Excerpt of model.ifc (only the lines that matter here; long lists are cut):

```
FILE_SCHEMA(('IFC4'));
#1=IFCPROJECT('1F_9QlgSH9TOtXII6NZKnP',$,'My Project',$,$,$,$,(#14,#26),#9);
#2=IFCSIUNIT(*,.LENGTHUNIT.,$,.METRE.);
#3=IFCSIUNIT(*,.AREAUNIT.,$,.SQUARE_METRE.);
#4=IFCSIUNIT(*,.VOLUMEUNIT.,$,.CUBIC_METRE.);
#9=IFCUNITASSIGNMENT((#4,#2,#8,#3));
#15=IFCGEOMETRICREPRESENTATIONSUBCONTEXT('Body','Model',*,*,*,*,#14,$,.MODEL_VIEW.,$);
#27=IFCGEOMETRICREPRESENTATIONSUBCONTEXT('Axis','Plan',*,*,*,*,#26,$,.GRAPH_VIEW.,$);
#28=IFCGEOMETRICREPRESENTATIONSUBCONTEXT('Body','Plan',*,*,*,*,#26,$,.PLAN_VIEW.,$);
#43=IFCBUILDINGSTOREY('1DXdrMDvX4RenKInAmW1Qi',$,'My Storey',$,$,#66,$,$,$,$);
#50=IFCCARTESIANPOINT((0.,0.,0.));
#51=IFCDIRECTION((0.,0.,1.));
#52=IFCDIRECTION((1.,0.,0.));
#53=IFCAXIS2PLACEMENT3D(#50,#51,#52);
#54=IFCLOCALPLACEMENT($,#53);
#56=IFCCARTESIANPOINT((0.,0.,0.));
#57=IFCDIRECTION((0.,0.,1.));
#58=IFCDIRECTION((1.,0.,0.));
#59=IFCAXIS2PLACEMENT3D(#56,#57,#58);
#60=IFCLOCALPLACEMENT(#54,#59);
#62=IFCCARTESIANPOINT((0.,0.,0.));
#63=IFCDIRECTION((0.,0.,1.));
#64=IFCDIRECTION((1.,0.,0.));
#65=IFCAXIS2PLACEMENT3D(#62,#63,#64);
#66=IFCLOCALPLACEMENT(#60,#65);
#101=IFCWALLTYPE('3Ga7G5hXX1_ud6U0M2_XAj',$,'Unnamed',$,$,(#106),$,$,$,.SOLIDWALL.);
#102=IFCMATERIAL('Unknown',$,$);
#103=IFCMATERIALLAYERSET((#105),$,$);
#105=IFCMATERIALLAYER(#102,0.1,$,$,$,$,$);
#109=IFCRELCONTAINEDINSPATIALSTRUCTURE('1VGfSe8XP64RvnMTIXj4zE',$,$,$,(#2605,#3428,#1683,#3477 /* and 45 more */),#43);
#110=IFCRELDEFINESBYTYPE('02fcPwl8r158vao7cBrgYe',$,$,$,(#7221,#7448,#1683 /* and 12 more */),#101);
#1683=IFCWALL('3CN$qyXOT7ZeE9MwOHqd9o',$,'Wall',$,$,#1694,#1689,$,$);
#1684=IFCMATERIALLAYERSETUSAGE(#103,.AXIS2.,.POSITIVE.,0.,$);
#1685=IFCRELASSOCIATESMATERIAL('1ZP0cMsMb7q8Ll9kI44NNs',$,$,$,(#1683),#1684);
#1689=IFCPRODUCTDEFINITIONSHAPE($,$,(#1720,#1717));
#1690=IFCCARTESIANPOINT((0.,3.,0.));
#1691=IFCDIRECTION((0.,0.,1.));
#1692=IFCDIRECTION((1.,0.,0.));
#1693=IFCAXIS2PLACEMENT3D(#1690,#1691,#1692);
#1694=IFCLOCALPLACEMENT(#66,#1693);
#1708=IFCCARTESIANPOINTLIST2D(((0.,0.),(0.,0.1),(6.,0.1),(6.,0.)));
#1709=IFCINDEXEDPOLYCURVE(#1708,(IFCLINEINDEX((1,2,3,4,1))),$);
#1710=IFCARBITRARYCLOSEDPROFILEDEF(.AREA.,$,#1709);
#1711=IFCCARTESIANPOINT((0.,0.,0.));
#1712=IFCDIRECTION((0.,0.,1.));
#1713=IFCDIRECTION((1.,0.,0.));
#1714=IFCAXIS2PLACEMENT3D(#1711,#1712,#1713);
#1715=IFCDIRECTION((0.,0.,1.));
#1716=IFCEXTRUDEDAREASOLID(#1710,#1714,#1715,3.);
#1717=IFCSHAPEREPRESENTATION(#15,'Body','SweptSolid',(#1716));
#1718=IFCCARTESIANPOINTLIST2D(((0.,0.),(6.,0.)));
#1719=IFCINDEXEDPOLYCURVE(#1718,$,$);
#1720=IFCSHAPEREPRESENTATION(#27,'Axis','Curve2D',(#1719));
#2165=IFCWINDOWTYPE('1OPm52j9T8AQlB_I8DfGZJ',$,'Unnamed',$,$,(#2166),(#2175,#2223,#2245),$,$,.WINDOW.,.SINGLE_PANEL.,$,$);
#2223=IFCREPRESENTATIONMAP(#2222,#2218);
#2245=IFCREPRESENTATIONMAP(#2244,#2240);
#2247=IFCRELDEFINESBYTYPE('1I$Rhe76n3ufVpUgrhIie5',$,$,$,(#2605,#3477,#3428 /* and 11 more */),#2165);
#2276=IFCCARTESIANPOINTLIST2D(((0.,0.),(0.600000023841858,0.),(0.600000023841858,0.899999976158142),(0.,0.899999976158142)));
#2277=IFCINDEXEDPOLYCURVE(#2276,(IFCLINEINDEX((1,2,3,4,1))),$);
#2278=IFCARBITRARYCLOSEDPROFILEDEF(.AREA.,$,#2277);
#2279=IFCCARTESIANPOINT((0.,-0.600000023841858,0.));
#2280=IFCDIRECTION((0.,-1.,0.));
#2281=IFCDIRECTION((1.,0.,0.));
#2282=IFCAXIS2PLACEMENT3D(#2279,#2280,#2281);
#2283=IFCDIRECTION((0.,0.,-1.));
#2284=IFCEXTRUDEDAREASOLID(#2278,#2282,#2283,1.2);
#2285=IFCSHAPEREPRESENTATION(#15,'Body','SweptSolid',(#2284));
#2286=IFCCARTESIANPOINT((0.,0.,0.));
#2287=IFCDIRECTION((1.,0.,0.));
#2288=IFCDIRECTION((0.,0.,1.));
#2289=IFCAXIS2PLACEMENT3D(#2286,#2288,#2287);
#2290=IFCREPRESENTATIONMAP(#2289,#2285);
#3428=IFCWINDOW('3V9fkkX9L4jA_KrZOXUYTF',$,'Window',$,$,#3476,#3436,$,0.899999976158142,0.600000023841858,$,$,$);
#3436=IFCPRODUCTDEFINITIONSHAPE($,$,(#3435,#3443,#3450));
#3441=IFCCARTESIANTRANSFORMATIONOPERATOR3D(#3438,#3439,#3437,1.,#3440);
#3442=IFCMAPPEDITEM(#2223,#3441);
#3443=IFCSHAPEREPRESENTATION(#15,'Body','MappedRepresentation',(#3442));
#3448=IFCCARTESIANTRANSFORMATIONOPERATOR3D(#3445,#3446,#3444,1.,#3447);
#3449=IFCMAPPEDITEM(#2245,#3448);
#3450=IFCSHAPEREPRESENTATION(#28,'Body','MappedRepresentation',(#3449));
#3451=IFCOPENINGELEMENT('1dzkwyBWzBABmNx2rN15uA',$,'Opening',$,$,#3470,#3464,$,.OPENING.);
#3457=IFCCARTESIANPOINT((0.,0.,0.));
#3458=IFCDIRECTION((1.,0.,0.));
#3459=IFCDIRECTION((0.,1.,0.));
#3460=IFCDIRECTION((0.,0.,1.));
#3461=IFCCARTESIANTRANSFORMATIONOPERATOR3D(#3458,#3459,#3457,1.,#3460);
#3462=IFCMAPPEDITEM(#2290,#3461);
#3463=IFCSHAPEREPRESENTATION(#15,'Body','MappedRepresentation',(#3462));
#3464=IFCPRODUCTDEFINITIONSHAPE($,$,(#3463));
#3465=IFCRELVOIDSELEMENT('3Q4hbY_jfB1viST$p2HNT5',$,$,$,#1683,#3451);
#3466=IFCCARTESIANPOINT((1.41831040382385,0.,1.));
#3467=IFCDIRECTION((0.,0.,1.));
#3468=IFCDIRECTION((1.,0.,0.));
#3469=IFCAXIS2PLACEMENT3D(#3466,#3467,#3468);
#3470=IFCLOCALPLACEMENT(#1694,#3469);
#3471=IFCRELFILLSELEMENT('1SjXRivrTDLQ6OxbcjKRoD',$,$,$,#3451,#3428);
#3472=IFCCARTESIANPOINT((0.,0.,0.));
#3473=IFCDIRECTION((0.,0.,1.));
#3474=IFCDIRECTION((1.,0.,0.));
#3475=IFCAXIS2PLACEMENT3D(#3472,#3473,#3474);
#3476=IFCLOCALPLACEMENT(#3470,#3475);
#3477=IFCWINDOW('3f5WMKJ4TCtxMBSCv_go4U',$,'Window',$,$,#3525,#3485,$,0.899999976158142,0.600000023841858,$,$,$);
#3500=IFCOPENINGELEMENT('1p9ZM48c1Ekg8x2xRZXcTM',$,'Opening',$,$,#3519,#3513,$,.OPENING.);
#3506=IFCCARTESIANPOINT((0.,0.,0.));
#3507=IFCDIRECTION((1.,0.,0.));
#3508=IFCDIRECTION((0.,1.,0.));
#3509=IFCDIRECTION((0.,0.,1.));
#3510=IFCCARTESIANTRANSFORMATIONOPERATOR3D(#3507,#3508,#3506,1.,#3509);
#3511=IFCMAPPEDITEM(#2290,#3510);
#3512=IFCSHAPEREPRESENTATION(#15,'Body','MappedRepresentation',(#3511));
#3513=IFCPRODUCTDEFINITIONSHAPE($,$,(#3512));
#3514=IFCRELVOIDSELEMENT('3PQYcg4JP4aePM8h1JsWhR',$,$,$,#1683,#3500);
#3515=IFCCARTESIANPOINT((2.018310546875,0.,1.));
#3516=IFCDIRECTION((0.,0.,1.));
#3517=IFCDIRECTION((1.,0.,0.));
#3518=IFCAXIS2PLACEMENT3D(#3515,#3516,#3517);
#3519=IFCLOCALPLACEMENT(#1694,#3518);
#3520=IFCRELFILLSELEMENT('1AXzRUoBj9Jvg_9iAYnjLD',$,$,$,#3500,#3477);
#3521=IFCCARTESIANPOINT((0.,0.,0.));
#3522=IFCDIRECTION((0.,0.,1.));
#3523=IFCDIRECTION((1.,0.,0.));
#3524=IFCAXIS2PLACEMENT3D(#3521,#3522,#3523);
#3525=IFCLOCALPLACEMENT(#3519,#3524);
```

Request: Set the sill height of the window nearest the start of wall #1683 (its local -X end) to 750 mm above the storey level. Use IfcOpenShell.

```python
import numpy as np
import ifcopenshell
import ifcopenshell.api.geometry
import ifcopenshell.geom
import ifcopenshell.util.element
import ifcopenshell.util.placement
import ifcopenshell.util.shape
import ifcopenshell.util.unit

model = ifcopenshell.open("model.ifc")
unit_scale = ifcopenshell.util.unit.calculate_unit_scale(model)

window = model.by_id(3428)
opening = window.FillsVoids[0].RelatingOpeningElement
storey = ifcopenshell.util.element.get_container(window, ifc_class="IfcBuildingStorey")
level = ifcopenshell.util.placement.get_local_placement(storey.ObjectPlacement)[2, 3]

# The opening's origin need not be at the sill, so measure its lowest point.
shape = ifcopenshell.geom.create_shape(ifcopenshell.geom.settings(), opening)
bottom = ifcopenshell.util.shape.get_shape_bottom_elevation(shape, shape.geometry) / unit_scale
dz = level + 0.75 / unit_scale - bottom

shift = np.array([0.0, 0.0, dz])
# The window is placed relative to its opening, so it follows when the opening moves.
matrix = ifcopenshell.util.placement.get_local_placement(opening.ObjectPlacement)
matrix[:3, 3] += shift
ifcopenshell.api.geometry.edit_object_placement(
    model, product=opening, matrix=matrix, is_si=False, should_transform_children=True
)

print(f"moved by {dz * unit_scale:+.3f} m")

model.write("model_edited.ifc")
```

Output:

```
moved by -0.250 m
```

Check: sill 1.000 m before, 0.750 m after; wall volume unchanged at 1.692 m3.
